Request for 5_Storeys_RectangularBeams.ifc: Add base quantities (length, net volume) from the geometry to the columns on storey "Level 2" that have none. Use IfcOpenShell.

First a look at what the model holds.

```python
import ifcopenshell
import ifcopenshell.util.element
import ifcopenshell.util.unit

model = ifcopenshell.open("5_Storeys_RectangularBeams.ifc")
print(model.schema)
for unit_type in ("LENGTHUNIT", "AREAUNIT", "VOLUMEUNIT"):
    print(unit_type, ifcopenshell.util.unit.calculate_unit_scale(model, unit_type))
storey = next(s for s in model.by_type("IfcBuildingStorey") if s.Name == "Level 2")
columns = [e for e in ifcopenshell.util.element.get_decomposition(storey) if e.is_a("IfcColumn")]
for e in sorted(columns, key=lambda e: e.id()):
    print(e.id(), e.is_a(), e.Name, list(ifcopenshell.util.element.get_psets(e, qtos_only=True)), sep=" | ")
```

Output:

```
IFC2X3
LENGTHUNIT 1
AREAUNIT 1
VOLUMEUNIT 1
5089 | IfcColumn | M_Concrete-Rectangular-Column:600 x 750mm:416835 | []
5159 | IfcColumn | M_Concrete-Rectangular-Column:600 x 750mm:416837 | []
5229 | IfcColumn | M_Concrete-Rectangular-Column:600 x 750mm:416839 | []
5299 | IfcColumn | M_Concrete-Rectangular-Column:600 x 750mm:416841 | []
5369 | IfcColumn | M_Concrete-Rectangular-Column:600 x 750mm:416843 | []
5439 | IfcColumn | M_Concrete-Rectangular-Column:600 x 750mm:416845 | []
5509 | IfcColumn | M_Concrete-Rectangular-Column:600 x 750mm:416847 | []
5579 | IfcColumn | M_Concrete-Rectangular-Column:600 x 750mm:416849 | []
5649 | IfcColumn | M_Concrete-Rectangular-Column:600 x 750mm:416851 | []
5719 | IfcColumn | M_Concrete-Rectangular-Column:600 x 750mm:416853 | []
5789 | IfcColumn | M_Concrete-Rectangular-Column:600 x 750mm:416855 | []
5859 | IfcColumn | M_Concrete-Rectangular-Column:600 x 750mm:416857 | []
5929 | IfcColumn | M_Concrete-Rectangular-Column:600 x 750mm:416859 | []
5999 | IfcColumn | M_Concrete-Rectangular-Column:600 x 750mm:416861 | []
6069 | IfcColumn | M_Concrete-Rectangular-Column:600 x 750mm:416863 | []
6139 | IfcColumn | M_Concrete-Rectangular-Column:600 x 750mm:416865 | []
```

```python
import ifcopenshell
import ifcopenshell.api.pset
import ifcopenshell.geom
import ifcopenshell.util.element
import ifcopenshell.util.shape
import ifcopenshell.util.unit

model = ifcopenshell.open("5_Storeys_RectangularBeams.ifc")
unit_scale = ifcopenshell.util.unit.calculate_unit_scale(model)
volume_scale = ifcopenshell.util.unit.calculate_unit_scale(model, "VOLUMEUNIT")
settings = ifcopenshell.geom.settings()

storey = next(s for s in model.by_type("IfcBuildingStorey") if s.Name == "Level 2")
columns = [e for e in ifcopenshell.util.element.get_decomposition(storey) if e.is_a("IfcColumn")]

for e in sorted(columns, key=lambda e: e.id()):
    if ifcopenshell.util.element.get_psets(e, qtos_only=True, should_inherit=False):
        continue
    # Geometry comes back in metres, in the element's own axes.
    shape = ifcopenshell.geom.create_shape(settings, e)
    values = {
        "Length": ifcopenshell.util.shape.get_z(shape.geometry) / unit_scale,
        "NetVolume": ifcopenshell.util.shape.get_volume(shape.geometry) / volume_scale,
    }
    qto = ifcopenshell.api.pset.add_qto(model, product=e, name="BaseQuantities")
    ifcopenshell.api.pset.edit_qto(model, qto=qto, properties=values)
    print(e.id(), {k: round(v, 3) for k, v in values.items()})

model.write("5_Storeys_RectangularBeams_rev.ifc")
```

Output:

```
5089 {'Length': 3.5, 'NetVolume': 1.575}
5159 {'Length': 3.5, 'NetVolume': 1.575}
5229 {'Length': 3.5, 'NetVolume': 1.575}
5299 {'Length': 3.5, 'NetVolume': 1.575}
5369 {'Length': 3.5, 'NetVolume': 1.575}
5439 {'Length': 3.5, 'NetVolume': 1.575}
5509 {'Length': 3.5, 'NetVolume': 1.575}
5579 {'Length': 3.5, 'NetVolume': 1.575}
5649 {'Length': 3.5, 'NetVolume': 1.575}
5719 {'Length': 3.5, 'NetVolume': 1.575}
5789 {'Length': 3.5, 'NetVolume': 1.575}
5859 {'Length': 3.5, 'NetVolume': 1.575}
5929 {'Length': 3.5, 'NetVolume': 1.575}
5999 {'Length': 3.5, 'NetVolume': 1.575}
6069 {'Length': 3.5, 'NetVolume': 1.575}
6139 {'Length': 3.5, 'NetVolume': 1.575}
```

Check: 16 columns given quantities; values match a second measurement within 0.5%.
